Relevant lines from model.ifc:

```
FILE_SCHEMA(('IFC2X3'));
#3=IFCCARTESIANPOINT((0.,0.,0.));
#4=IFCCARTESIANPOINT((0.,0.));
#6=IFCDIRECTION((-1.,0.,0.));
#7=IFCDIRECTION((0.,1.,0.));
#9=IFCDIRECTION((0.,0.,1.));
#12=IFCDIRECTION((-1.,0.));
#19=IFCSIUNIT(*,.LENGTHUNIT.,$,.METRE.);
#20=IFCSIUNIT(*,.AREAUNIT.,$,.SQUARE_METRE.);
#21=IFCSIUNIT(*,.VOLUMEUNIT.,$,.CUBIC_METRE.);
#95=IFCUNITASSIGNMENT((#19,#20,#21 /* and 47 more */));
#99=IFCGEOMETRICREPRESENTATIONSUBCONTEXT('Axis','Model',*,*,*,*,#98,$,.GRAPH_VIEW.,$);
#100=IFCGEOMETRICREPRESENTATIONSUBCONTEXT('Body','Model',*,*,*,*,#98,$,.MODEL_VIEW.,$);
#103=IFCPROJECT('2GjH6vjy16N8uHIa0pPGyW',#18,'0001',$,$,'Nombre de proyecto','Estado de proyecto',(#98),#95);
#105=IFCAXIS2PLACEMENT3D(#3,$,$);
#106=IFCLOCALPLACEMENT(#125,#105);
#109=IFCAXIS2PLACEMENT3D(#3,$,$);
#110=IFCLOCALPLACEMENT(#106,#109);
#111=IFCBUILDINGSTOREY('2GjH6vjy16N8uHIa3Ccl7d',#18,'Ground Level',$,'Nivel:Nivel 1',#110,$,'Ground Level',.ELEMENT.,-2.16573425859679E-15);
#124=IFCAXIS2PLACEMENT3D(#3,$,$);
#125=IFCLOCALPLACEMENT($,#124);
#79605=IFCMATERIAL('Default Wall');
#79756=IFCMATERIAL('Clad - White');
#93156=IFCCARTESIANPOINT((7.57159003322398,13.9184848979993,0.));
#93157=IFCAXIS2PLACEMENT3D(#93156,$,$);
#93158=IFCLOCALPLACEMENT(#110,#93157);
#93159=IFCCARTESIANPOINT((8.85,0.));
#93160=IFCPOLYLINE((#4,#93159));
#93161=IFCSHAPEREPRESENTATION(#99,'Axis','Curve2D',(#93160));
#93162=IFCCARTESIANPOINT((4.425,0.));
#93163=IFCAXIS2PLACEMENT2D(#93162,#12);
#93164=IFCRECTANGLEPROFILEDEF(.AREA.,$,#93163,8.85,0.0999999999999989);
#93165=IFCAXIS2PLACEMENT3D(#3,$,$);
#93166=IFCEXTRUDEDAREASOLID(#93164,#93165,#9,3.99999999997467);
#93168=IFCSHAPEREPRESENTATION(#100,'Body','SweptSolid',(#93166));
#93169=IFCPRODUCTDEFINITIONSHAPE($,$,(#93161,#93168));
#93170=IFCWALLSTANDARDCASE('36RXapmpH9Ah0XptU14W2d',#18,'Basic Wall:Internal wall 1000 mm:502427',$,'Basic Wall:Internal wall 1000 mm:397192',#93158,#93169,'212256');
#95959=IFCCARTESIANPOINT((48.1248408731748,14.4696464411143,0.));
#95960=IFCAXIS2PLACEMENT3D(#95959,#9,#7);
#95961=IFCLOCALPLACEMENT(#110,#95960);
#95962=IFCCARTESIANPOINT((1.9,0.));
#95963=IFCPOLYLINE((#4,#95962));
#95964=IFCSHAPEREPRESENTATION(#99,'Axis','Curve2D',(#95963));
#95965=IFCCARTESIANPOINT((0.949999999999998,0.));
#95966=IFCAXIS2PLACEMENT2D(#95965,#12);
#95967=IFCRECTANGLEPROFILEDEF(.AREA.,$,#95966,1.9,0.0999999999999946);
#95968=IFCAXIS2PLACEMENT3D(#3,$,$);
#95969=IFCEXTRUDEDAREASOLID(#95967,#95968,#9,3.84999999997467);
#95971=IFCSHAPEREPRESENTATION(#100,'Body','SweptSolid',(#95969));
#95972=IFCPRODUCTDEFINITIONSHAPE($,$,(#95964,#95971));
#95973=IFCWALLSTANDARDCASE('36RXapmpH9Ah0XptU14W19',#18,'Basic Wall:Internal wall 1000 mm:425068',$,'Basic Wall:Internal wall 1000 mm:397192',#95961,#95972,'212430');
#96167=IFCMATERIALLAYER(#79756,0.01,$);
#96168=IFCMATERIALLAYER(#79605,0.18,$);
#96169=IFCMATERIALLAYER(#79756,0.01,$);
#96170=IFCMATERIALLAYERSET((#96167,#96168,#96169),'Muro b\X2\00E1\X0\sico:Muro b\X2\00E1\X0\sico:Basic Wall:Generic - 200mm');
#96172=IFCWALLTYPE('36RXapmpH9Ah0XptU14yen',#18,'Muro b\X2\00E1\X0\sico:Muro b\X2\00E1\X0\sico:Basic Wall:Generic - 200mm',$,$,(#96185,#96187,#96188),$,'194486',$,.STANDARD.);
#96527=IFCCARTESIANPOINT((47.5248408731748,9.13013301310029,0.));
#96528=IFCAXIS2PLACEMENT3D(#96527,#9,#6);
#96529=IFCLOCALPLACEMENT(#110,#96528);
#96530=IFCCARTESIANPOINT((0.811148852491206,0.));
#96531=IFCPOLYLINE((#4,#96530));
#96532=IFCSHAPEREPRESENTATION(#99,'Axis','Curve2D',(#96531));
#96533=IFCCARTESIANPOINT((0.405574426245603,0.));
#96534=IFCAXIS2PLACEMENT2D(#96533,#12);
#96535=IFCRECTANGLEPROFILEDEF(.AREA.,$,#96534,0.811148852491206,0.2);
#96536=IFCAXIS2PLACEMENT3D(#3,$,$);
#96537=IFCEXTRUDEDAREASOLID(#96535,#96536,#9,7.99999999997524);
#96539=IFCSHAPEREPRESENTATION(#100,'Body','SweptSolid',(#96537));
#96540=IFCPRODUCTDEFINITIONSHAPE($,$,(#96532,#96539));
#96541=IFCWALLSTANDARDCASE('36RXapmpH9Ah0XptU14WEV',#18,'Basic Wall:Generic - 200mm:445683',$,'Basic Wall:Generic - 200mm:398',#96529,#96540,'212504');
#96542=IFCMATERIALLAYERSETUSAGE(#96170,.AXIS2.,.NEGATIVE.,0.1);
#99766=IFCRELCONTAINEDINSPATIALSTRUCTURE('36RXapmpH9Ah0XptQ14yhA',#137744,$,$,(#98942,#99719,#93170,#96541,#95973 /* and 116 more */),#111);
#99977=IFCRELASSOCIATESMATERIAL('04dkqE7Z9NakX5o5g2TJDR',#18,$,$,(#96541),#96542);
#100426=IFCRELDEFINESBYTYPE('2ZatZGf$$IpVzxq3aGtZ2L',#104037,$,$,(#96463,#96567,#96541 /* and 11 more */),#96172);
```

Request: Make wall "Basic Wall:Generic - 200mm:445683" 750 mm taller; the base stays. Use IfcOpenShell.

```python
import ifcopenshell
import ifcopenshell.geom
import ifcopenshell.util.representation
import ifcopenshell.util.shape

model = ifcopenshell.open("model.ifc")
settings = ifcopenshell.geom.settings()


def volume(element):
    """Net volume in cubic metres, openings subtracted."""
    shape = ifcopenshell.geom.create_shape(settings, element)
    return ifcopenshell.util.shape.get_volume(shape.geometry)


wall = model.by_guid("36RXapmpH9Ah0XptU14WEV")
before = volume(wall)

body = ifcopenshell.util.representation.get_representation(wall, "Model", "Body")
solid = body.Items[0]
old_height = solid.Depth
solid.Depth += 0.75
after = volume(wall)

print(f"height {old_height:g} -> {solid.Depth:g}, volume {before:.3f} -> {after:.3f} m3")

model.write("model_edited.ifc")
```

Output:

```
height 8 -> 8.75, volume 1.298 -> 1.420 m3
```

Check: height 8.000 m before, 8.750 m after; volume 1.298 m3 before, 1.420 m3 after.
